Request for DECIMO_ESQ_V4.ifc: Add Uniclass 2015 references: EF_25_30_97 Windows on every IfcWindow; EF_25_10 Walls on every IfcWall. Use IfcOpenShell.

First a look at what the model holds.

```python
import ifcopenshell

model = ifcopenshell.open("DECIMO_ESQ_V4.ifc")
print(model.schema)
print("classifications:", [c.Name for c in model.by_type("IfcClassification")])
for ifc_class in ("IfcDoor", "IfcRoof", "IfcStair", "IfcWall", "IfcWindow"):
    print(ifc_class, len(model.by_type(ifc_class)))
```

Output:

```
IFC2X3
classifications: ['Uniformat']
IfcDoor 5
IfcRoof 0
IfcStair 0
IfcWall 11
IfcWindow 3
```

```python
import ifcopenshell
import ifcopenshell.api.classification

model = ifcopenshell.open("DECIMO_ESQ_V4.ifc")

# IFC2X3 requires Source and Edition and has no link from the project to the system.
system = model.create_entity("IfcClassification", Source="NBS", Edition="2015", Name="Uniclass 2015")

codes = {
    "IfcWindow": ("EF_25_30_97", "Windows"),
    "IfcWall": ("EF_25_10", "Walls"),
}
for ifc_class, (code, name) in codes.items():
    products = model.by_type(ifc_class)
    ifcopenshell.api.classification.add_reference(
        model, products=products, classification=system, identification=code, name=name
    )
    print(code, len(products))

model.write("DECIMO_ESQ_V4_v2.ifc")
```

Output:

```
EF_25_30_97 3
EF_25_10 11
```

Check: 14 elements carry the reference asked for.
